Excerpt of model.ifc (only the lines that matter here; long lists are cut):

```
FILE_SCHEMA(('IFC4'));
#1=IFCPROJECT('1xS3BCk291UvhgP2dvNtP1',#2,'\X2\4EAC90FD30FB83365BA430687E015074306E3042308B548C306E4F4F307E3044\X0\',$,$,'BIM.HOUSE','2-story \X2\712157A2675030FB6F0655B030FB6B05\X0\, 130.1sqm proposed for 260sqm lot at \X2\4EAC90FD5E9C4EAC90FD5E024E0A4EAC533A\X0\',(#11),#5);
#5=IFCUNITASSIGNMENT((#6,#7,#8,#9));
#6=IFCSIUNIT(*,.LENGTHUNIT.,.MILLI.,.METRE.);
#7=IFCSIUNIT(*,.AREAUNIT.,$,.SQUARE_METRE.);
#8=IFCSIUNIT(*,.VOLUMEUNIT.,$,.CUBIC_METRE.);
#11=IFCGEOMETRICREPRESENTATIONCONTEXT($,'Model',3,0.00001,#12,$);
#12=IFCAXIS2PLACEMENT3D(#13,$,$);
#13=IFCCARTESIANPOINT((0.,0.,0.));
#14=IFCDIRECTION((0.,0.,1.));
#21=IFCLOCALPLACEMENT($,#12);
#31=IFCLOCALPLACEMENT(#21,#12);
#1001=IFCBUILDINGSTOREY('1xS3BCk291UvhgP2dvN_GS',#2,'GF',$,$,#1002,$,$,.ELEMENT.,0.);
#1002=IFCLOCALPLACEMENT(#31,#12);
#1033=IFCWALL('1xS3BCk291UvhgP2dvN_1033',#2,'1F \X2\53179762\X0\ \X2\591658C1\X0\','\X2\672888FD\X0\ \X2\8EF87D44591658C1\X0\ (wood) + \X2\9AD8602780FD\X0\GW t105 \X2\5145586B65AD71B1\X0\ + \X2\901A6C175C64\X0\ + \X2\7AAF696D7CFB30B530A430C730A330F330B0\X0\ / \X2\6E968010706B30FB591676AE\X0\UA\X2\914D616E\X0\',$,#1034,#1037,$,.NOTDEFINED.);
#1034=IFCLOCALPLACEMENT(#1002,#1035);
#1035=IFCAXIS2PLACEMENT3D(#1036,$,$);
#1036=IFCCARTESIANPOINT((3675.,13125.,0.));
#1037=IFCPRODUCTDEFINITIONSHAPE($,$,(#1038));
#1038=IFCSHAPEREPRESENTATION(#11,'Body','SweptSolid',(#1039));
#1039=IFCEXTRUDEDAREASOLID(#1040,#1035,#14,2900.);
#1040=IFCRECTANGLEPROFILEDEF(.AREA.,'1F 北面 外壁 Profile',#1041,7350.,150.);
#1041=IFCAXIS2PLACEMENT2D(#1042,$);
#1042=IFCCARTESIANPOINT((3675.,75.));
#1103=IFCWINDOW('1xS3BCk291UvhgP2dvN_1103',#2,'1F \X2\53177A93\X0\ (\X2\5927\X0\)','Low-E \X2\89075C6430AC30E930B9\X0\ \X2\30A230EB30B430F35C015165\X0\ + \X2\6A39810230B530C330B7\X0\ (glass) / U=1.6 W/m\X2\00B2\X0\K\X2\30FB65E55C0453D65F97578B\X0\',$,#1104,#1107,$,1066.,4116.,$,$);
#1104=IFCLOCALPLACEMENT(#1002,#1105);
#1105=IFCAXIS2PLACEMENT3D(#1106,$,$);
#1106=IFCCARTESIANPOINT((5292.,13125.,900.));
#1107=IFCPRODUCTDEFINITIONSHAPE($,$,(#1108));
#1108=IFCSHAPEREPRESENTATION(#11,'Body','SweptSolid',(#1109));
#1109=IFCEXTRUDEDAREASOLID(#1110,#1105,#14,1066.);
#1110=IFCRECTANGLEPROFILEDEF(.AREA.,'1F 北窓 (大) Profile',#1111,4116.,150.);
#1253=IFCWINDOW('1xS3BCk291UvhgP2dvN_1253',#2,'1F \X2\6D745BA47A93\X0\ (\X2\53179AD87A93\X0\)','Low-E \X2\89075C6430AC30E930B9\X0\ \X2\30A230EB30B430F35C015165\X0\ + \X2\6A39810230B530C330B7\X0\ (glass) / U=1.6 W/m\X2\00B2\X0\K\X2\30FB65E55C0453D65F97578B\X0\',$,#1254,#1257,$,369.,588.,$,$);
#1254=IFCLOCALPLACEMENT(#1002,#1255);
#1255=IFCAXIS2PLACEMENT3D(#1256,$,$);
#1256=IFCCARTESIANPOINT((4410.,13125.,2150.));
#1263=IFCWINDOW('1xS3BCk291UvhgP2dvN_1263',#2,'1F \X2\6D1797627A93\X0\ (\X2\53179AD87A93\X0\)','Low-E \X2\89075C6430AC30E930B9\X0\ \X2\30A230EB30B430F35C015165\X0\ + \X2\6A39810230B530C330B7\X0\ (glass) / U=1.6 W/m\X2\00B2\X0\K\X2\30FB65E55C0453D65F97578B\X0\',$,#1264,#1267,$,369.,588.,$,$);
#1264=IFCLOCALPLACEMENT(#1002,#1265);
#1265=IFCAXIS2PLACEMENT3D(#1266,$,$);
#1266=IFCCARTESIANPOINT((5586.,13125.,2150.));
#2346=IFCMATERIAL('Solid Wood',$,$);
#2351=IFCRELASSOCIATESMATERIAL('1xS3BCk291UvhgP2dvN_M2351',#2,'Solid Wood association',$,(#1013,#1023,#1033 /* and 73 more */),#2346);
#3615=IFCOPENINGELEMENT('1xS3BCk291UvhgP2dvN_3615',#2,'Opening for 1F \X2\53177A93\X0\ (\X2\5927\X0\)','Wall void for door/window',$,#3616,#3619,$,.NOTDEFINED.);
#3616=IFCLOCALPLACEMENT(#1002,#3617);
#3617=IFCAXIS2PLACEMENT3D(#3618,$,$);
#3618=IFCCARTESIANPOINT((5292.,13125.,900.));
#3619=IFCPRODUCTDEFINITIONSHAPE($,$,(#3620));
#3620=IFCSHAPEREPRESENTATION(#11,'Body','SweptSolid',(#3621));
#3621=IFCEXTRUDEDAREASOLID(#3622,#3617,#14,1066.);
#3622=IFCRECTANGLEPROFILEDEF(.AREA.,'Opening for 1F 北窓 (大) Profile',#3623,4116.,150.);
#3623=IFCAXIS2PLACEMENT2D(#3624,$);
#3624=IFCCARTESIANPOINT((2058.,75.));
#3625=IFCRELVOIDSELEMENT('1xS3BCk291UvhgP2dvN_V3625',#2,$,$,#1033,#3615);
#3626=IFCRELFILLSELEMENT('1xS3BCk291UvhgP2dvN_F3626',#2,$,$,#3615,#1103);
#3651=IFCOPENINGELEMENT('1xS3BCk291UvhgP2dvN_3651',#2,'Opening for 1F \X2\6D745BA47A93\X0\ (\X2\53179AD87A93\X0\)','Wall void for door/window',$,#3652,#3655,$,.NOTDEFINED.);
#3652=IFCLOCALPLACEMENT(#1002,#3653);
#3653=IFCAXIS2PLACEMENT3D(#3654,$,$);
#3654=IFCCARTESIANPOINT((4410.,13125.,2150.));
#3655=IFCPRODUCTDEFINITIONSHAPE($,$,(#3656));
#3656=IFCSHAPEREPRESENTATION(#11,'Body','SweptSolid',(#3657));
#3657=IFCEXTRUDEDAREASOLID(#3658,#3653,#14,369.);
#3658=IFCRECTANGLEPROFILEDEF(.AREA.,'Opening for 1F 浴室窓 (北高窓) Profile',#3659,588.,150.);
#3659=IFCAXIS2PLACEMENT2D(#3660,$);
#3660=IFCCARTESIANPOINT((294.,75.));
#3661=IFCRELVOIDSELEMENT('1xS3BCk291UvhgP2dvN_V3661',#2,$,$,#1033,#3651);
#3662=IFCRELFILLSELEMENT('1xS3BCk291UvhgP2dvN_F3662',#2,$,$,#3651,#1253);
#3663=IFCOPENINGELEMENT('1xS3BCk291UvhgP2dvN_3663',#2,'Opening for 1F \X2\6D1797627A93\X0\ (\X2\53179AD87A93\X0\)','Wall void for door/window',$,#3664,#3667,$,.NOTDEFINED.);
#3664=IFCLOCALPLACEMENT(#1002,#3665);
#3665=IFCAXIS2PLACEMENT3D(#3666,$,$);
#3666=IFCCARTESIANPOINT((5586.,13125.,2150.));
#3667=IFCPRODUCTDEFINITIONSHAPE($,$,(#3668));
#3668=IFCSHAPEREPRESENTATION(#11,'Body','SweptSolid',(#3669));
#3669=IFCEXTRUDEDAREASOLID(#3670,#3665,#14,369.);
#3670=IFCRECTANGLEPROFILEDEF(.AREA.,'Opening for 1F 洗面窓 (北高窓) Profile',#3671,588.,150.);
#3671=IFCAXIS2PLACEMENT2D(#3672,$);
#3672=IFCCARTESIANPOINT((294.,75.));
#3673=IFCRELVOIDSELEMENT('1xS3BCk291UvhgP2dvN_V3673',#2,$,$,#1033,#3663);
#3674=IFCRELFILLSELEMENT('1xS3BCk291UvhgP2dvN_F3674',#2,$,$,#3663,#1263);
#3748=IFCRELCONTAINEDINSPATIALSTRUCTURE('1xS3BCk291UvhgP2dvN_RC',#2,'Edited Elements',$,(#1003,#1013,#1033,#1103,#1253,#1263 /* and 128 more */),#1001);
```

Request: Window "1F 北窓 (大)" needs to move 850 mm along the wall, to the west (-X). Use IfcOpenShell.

```python
import ifcopenshell
import ifcopenshell.api.geometry
import ifcopenshell.util.placement
import ifcopenshell.util.unit

model = ifcopenshell.open("model.ifc")
unit_scale = ifcopenshell.util.unit.calculate_unit_scale(model)

window = model.by_guid("1xS3BCk291UvhgP2dvN_1103")
opening = window.FillsVoids[0].RelatingOpeningElement
wall = opening.VoidsElements[0].RelatingBuildingElement

wall_matrix = ifcopenshell.util.placement.get_local_placement(wall.ObjectPlacement)
shift = wall_matrix[:3, 0] * -0.85 / unit_scale
before = ifcopenshell.util.placement.get_local_placement(window.ObjectPlacement)[:3, 3].copy()

# The window is not placed relative to its opening, so move both.
for product in (opening, window):
    matrix = ifcopenshell.util.placement.get_local_placement(product.ObjectPlacement)
    matrix[:3, 3] += shift
    ifcopenshell.api.geometry.edit_object_placement(model, product=product, matrix=matrix, is_si=False)

after = ifcopenshell.util.placement.get_local_placement(window.ObjectPlacement)[:3, 3]
print("window moved by", (after - before).round(3) + 0.0)

model.write("model_updated.ifc")
```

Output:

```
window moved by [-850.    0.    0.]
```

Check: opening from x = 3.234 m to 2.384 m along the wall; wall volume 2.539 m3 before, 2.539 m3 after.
